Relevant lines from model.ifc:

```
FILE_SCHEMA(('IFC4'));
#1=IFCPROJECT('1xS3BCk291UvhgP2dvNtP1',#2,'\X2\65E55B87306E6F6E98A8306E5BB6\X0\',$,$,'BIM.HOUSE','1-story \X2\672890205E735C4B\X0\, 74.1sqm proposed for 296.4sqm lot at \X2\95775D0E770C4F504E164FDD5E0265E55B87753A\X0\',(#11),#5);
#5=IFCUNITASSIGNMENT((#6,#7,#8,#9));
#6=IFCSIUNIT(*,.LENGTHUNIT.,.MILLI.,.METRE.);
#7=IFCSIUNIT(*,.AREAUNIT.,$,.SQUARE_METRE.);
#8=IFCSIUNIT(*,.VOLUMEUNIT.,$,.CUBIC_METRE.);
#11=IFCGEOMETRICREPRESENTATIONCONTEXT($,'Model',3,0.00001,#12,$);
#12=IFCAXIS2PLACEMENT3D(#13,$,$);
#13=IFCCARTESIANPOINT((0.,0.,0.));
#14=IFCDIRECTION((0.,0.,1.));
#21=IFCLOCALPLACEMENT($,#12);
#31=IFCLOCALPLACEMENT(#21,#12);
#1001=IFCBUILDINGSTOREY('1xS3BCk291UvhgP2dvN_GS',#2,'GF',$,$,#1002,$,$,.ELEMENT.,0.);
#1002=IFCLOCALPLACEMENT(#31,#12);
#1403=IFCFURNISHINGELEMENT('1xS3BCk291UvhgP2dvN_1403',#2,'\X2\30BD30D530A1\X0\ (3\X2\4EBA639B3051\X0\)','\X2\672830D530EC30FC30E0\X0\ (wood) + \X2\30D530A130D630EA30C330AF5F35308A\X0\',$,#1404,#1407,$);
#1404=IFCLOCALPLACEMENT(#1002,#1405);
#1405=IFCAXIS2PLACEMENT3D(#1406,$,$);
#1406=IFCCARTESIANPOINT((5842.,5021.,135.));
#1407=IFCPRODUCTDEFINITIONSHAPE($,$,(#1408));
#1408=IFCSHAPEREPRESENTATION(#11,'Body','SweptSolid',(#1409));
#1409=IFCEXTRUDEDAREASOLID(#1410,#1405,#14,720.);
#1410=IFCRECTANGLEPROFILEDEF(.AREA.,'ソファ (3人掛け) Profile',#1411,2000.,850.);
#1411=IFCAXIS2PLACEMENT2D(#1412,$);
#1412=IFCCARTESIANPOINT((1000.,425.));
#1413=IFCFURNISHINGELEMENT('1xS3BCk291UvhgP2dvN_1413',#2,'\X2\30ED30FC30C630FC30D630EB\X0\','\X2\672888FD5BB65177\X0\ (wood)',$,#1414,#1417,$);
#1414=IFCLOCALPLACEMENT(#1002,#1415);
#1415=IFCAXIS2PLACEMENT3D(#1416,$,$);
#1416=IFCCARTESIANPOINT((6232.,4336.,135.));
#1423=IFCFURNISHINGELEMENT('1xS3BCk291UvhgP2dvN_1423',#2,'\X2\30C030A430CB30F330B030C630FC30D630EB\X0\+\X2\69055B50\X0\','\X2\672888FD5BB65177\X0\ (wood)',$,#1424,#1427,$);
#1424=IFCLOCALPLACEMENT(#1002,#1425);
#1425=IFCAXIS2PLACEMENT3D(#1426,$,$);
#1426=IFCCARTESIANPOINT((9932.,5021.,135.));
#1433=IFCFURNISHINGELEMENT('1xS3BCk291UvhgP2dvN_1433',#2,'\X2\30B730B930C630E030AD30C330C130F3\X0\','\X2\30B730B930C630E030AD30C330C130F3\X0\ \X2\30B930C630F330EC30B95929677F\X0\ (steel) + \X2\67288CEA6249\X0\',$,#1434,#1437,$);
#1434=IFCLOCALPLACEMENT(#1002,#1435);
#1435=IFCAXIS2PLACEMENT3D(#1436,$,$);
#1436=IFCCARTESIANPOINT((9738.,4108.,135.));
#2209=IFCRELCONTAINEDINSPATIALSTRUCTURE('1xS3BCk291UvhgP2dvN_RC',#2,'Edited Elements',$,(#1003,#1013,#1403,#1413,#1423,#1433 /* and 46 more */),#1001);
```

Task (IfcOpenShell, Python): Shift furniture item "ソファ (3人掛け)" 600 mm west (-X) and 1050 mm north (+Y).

```python
import ifcopenshell
import ifcopenshell.api.geometry
import ifcopenshell.util.placement

model = ifcopenshell.open("model.ifc")

item = model.by_guid("1xS3BCk291UvhgP2dvN_1403")
matrix = ifcopenshell.util.placement.get_local_placement(item.ObjectPlacement)
matrix[0, 3] -= 600.0
matrix[1, 3] += 1050.0
ifcopenshell.api.geometry.edit_object_placement(model, product=item, matrix=matrix, is_si=False)

print(ifcopenshell.util.placement.get_local_placement(item.ObjectPlacement).round(3) + 0.0)

model.write("model_rev.ifc")
```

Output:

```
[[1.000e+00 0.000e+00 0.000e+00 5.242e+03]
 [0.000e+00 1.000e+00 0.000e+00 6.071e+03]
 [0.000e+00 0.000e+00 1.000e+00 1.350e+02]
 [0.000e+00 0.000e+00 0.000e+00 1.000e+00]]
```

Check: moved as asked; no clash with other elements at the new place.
